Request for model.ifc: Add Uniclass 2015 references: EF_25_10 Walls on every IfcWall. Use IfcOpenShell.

First a look at what the model holds.

```python
import ifcopenshell

model = ifcopenshell.open("model.ifc")
print(model.schema)
print("classifications:", [c.Name for c in model.by_type("IfcClassification")])
for ifc_class in ("IfcDoor", "IfcRoof", "IfcStair", "IfcWall", "IfcWindow"):
    print(ifc_class, len(model.by_type(ifc_class)))
```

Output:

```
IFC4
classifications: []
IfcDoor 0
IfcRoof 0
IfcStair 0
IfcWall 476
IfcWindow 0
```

```python
import ifcopenshell
import ifcopenshell.api.classification

model = ifcopenshell.open("model.ifc")

system = ifcopenshell.api.classification.add_classification(model, classification="Uniclass 2015")

codes = {
    "IfcWall": ("EF_25_10", "Walls"),
}
for ifc_class, (code, name) in codes.items():
    products = model.by_type(ifc_class)
    ifcopenshell.api.classification.add_reference(
        model, products=products, classification=system, identification=code, name=name
    )
    print(code, len(products))

model.write("model_edited.ifc")
```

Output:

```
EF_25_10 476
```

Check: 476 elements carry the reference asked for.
